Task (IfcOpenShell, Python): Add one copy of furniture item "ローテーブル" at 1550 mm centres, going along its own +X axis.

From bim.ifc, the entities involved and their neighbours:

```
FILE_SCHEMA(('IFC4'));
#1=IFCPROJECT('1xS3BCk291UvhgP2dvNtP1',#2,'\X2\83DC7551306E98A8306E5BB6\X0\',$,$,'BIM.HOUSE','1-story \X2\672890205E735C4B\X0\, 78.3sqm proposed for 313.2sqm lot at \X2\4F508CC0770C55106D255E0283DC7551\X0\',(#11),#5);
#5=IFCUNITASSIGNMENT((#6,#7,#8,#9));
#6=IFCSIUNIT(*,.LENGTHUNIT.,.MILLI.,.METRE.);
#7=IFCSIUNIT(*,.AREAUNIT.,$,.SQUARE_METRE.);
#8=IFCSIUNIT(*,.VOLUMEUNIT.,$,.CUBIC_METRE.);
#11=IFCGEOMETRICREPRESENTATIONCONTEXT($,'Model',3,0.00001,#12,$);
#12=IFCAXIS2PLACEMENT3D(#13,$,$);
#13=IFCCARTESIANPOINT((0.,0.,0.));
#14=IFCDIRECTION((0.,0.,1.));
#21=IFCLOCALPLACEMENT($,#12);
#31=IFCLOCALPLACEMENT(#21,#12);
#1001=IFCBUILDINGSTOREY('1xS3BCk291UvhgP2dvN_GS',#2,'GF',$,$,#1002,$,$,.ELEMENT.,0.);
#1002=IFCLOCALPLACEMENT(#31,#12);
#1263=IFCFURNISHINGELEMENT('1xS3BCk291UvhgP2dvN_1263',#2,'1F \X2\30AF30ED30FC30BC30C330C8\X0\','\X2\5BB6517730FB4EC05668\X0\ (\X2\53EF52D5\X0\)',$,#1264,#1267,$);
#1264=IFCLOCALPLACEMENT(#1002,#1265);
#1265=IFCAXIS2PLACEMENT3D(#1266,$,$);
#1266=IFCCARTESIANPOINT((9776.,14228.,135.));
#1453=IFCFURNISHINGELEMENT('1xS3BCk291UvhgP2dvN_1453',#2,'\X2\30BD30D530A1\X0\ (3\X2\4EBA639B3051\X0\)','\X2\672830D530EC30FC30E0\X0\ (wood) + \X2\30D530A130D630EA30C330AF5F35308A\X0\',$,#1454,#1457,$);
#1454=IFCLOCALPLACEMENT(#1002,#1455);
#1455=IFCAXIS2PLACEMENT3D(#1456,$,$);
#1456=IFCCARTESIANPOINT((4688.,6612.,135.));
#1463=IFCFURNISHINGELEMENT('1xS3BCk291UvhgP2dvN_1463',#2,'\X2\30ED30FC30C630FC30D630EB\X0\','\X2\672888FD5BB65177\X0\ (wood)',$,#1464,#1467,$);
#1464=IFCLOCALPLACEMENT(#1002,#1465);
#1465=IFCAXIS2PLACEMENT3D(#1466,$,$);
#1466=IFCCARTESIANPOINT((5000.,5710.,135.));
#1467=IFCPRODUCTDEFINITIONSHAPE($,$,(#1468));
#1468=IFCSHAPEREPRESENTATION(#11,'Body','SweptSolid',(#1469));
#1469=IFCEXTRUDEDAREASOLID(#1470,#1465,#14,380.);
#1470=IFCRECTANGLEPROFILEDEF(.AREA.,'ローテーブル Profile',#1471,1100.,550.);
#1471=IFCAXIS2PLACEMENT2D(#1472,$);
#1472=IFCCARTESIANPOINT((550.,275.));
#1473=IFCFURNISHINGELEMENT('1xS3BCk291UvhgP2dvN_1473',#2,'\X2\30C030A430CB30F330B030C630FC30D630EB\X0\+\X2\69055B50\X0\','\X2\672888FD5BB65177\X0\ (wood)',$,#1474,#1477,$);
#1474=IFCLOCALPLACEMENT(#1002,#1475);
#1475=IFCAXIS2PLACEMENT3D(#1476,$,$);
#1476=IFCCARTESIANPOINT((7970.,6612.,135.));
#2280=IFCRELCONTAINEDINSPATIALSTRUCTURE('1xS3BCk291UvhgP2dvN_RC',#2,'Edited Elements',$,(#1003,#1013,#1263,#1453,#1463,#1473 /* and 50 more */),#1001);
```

```python
import ifcopenshell
import ifcopenshell.api.geometry
import ifcopenshell.api.root
import ifcopenshell.util.element
import ifcopenshell.util.placement

model = ifcopenshell.open("bim.ifc")


def reuse_history(source, copy):
    """copy_class also copies each property set's owner history, people and application; keep the originals."""
    for rel in copy.IsDefinedBy:
        if rel.is_a("IfcRelDefinesByProperties") and (history := rel.RelatingPropertyDefinition.OwnerHistory):
            rel.RelatingPropertyDefinition.OwnerHistory = source.OwnerHistory
            ifcopenshell.util.element.remove_deep2(model, history)


source = model.by_id(1463)
base = ifcopenshell.util.placement.get_local_placement(source.ObjectPlacement)
step = base[:3, 0] * 1550.0

for i in range(1, 2):
    copy = ifcopenshell.api.root.copy_class(model, product=source)
    copy.Representation = ifcopenshell.util.element.copy_deep(
        model, source.Representation, exclude=["IfcGeometricRepresentationContext", "IfcRepresentationMap"]
    )
    reuse_history(source, copy)
    matrix = base.copy()
    matrix[:3, 3] += i * step
    print("added at", matrix[:3, 3].round(3) + 0.0)
    ifcopenshell.api.geometry.edit_object_placement(model, product=copy, matrix=matrix, is_si=False)

model.write("bim_updated.ifc")
```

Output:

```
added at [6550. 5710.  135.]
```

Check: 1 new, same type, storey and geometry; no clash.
